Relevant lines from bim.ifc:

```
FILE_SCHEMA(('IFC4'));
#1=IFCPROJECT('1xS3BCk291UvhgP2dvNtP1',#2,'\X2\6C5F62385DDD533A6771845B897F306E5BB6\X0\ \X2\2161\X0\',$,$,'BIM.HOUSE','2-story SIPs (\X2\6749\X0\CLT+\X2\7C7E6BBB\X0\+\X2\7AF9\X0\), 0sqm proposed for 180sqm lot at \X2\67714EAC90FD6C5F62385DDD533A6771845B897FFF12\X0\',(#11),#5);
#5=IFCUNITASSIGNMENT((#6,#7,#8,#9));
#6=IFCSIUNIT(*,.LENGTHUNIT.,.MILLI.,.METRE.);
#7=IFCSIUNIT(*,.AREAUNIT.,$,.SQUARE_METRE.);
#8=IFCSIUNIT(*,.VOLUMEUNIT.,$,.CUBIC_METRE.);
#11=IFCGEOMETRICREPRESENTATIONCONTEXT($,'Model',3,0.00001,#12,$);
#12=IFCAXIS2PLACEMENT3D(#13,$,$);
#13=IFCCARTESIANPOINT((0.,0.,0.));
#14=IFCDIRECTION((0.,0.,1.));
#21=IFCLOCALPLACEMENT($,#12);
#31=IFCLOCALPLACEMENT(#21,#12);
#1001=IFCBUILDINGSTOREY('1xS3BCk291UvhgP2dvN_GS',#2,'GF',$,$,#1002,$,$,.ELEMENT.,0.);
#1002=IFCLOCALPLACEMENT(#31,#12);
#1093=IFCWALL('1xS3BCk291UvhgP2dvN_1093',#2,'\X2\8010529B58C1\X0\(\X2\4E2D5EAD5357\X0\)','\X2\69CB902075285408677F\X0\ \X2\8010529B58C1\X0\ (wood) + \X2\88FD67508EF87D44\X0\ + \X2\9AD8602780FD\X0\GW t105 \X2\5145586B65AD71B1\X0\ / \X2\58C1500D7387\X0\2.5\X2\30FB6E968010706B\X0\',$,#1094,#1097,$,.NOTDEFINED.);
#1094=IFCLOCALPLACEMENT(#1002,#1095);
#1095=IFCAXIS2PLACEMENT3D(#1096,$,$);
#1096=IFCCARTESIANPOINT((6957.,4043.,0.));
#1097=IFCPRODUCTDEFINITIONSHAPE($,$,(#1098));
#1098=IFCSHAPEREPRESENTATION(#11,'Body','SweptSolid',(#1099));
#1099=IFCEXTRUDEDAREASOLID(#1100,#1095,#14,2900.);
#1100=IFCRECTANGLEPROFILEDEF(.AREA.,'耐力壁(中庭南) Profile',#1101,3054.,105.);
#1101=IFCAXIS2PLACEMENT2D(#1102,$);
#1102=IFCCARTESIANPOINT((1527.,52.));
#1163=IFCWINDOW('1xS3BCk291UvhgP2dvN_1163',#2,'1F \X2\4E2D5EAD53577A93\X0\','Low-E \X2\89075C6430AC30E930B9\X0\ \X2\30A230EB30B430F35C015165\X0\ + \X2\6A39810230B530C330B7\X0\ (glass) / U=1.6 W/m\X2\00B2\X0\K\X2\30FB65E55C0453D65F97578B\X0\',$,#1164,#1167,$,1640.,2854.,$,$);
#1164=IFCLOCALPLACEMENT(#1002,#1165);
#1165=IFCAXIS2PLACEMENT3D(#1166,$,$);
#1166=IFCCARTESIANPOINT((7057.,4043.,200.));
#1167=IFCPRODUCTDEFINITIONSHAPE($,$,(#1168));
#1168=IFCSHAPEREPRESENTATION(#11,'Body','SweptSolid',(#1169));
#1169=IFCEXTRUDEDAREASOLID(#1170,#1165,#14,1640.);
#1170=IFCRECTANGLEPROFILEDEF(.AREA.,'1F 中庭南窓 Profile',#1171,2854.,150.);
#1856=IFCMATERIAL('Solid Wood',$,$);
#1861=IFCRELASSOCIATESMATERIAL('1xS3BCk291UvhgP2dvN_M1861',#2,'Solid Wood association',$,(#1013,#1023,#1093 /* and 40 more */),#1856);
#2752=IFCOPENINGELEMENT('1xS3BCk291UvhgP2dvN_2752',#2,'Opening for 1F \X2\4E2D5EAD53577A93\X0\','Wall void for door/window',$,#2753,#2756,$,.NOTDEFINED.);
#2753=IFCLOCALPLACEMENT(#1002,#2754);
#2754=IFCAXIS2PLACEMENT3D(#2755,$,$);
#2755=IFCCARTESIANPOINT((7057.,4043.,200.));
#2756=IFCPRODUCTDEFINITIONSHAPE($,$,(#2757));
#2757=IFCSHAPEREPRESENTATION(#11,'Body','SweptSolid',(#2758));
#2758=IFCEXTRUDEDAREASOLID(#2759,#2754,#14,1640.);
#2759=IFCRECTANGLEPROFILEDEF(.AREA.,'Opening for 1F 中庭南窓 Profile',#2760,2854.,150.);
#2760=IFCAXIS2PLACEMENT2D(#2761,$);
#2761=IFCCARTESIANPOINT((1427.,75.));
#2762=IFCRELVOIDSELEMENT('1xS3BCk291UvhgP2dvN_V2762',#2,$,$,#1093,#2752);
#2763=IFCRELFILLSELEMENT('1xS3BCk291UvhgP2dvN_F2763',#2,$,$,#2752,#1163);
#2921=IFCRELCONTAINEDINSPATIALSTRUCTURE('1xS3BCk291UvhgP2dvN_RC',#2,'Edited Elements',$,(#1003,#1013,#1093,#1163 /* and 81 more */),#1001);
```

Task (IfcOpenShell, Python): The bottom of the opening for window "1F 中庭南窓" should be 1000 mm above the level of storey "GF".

```python
import numpy as np
import ifcopenshell
import ifcopenshell.api.geometry
import ifcopenshell.geom
import ifcopenshell.util.element
import ifcopenshell.util.placement
import ifcopenshell.util.shape
import ifcopenshell.util.unit

model = ifcopenshell.open("bim.ifc")
unit_scale = ifcopenshell.util.unit.calculate_unit_scale(model)

window = model.by_guid("1xS3BCk291UvhgP2dvN_1163")
opening = window.FillsVoids[0].RelatingOpeningElement
storey = ifcopenshell.util.element.get_container(window, ifc_class="IfcBuildingStorey")
level = ifcopenshell.util.placement.get_local_placement(storey.ObjectPlacement)[2, 3]

# The opening's origin need not be at the sill, so measure its lowest point.
shape = ifcopenshell.geom.create_shape(ifcopenshell.geom.settings(), opening)
bottom = ifcopenshell.util.shape.get_shape_bottom_elevation(shape, shape.geometry) / unit_scale
dz = level + 1000.0 - bottom

shift = np.array([0.0, 0.0, dz])
# The window is not placed relative to its opening, so move both.
for product in (opening, window):
    matrix = ifcopenshell.util.placement.get_local_placement(product.ObjectPlacement)
    matrix[:3, 3] += shift
    ifcopenshell.api.geometry.edit_object_placement(model, product=product, matrix=matrix, is_si=False)

print(f"moved by {dz * unit_scale:+.3f} m")

model.write("bim_rev.ifc")
```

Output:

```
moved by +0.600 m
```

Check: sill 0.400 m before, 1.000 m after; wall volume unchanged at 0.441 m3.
